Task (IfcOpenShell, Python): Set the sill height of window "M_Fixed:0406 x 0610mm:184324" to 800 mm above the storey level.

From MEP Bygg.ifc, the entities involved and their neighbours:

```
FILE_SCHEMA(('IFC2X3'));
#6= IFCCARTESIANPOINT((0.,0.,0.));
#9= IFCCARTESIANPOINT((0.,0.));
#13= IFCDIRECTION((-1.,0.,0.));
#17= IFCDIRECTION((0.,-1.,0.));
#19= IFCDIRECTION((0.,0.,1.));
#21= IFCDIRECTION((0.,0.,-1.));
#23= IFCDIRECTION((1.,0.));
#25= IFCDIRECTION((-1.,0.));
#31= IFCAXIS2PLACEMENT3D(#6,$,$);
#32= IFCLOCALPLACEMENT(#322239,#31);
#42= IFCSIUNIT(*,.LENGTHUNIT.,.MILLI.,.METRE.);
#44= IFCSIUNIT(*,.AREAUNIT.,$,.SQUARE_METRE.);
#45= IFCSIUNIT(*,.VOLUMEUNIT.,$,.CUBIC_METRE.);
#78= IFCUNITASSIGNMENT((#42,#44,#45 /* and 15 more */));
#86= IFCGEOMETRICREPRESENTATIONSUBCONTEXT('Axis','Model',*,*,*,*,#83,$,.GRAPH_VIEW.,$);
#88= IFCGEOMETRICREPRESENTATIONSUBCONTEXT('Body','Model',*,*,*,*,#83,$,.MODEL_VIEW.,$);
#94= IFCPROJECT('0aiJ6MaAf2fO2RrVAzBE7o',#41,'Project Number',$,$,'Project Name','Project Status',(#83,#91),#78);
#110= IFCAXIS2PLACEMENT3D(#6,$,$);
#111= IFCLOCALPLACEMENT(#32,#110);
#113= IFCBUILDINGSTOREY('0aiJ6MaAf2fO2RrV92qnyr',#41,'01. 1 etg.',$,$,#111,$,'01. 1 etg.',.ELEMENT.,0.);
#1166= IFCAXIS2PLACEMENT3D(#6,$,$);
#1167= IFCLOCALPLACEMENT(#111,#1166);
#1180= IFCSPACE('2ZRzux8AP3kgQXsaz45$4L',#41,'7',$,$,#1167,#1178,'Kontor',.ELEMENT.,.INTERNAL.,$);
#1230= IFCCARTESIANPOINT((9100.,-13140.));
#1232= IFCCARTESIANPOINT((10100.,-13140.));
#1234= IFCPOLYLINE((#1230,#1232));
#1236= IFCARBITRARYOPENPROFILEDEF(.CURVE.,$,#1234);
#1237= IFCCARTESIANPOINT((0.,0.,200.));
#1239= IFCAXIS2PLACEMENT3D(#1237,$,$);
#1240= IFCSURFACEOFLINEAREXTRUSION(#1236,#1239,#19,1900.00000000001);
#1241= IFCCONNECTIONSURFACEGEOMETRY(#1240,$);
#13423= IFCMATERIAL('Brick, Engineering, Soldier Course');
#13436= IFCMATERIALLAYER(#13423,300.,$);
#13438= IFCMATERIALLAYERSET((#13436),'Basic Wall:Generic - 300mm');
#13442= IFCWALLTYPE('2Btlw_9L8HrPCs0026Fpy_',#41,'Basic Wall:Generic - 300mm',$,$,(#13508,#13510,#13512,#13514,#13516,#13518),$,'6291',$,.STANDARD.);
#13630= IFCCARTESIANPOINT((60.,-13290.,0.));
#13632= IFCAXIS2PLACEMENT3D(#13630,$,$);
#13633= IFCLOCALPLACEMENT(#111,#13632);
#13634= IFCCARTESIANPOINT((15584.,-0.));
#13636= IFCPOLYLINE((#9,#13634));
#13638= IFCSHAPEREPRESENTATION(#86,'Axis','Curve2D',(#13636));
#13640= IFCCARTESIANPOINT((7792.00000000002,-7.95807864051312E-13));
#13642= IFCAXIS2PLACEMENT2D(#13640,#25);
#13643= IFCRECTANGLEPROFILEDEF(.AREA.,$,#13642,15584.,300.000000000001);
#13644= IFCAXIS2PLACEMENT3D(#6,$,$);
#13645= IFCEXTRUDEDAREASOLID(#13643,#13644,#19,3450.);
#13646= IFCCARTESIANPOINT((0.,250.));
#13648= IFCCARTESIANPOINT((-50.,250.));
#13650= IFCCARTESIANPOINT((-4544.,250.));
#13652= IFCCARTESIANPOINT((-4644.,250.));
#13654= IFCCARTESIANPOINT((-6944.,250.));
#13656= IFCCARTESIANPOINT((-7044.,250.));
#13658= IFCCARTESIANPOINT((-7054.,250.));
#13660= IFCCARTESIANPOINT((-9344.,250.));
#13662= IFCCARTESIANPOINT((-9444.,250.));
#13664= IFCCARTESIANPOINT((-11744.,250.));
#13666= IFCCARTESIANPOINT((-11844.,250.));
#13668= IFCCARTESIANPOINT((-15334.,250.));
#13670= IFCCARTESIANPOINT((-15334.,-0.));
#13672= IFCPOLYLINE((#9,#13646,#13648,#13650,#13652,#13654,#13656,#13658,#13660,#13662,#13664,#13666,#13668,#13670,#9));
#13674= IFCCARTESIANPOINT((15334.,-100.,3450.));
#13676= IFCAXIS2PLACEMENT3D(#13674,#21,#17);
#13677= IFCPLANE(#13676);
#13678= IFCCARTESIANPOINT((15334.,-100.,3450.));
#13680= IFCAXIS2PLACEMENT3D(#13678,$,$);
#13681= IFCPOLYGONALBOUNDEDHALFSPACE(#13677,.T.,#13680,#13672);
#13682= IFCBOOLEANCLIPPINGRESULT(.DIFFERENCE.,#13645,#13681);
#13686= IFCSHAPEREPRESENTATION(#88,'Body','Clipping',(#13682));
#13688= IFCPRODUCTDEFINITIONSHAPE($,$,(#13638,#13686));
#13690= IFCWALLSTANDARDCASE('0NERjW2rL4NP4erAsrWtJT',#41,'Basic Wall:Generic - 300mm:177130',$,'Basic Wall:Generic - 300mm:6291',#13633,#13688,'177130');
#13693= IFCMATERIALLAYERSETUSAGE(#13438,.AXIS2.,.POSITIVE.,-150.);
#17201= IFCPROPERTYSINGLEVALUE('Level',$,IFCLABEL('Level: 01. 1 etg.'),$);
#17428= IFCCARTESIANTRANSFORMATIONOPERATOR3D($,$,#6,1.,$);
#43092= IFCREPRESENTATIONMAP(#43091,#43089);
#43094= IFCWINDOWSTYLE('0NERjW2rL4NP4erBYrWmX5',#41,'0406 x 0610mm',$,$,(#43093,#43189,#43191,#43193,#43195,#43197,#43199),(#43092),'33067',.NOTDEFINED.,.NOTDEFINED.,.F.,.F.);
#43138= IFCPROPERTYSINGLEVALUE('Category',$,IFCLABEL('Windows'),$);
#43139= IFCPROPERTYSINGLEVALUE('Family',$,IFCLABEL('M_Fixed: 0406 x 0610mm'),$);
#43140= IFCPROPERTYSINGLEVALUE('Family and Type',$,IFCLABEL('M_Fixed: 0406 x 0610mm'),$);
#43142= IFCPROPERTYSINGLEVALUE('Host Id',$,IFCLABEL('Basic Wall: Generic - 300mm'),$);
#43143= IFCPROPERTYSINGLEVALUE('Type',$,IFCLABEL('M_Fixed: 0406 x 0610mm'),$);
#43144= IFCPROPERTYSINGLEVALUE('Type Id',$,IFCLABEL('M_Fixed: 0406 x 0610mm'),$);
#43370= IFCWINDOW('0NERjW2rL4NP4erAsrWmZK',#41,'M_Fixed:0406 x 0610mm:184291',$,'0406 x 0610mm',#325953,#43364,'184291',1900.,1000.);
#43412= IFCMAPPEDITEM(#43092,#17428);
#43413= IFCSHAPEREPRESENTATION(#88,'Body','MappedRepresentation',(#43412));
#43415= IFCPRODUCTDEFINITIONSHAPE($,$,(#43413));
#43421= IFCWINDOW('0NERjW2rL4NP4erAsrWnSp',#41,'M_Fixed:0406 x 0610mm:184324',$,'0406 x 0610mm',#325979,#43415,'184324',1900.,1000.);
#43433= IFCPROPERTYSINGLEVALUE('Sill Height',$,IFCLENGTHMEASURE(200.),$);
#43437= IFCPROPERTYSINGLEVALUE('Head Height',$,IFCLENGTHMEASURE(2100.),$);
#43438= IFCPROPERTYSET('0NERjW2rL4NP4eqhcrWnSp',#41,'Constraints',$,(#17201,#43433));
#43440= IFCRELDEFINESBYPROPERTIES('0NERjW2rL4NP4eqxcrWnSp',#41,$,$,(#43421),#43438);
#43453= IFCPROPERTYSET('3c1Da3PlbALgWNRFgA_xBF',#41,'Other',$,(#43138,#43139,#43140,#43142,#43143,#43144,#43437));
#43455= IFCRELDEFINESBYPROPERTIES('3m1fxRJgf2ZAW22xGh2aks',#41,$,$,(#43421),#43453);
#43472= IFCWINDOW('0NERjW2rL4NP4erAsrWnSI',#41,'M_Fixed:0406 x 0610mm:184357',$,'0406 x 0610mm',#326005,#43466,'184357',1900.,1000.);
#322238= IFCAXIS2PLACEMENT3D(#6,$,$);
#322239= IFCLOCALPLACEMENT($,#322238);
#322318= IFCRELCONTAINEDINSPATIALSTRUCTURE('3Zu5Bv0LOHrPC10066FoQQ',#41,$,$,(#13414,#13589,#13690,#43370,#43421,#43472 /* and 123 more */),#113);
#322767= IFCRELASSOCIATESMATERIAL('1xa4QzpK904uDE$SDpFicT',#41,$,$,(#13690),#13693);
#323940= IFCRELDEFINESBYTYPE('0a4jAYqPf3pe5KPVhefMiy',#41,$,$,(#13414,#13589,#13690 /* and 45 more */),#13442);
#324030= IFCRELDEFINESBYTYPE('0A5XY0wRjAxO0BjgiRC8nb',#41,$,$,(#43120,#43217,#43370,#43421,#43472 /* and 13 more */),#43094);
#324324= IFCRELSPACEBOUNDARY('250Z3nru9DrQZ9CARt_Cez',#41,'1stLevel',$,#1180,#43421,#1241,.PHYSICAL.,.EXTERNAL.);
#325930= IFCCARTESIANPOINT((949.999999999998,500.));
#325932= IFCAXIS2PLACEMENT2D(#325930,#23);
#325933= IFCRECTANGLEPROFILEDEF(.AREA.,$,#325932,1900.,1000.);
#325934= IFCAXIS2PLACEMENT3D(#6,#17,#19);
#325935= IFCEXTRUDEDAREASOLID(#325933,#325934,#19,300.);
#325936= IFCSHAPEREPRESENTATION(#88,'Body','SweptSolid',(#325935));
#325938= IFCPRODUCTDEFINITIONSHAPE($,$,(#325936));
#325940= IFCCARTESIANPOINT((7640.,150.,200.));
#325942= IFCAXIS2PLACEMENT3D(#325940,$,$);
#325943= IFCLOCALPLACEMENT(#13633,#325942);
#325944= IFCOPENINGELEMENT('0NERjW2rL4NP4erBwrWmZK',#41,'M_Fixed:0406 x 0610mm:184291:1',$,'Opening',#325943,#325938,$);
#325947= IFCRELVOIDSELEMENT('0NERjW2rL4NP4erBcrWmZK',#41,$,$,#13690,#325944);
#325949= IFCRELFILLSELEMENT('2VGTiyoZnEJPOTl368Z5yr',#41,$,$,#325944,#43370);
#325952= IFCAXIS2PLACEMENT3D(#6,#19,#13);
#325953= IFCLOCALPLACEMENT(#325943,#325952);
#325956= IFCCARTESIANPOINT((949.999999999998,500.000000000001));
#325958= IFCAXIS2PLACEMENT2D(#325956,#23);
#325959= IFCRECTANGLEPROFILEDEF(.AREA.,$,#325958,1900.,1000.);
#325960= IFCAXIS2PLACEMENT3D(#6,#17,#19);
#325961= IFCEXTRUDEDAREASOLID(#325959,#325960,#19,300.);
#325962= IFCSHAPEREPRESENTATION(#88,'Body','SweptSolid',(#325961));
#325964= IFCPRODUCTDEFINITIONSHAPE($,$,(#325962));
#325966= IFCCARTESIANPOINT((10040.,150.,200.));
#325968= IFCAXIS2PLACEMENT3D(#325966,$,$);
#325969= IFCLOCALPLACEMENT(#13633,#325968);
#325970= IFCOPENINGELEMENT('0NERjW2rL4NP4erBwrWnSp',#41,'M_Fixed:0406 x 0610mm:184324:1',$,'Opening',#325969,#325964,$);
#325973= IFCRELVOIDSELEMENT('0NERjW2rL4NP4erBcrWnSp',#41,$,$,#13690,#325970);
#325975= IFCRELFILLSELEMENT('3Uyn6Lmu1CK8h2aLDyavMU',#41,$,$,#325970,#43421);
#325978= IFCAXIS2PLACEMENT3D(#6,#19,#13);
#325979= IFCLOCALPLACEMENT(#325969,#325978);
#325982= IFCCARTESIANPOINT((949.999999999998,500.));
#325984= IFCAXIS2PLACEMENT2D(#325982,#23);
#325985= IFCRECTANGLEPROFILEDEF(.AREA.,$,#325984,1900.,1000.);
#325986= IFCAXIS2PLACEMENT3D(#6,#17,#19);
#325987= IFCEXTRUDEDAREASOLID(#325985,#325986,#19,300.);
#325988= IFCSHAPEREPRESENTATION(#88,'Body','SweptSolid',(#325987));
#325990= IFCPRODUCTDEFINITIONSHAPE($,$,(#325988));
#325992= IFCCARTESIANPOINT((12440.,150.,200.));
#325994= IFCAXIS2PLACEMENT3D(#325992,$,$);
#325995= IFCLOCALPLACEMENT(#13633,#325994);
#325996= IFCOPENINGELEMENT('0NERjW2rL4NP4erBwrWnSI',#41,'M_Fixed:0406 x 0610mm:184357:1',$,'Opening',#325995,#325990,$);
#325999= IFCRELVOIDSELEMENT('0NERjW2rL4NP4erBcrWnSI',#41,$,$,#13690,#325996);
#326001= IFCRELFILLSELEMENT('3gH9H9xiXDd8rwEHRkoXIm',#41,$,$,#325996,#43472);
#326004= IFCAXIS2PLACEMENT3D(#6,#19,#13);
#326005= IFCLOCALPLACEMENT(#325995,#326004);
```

```python
import numpy as np
import ifcopenshell
import ifcopenshell.api.geometry
import ifcopenshell.api.pset
import ifcopenshell.geom
import ifcopenshell.util.element
import ifcopenshell.util.placement
import ifcopenshell.util.shape
import ifcopenshell.util.unit

model = ifcopenshell.open("MEP Bygg.ifc")
unit_scale = ifcopenshell.util.unit.calculate_unit_scale(model)

window = model.by_guid("0NERjW2rL4NP4erAsrWnSp")
opening = window.FillsVoids[0].RelatingOpeningElement
storey = ifcopenshell.util.element.get_container(window, ifc_class="IfcBuildingStorey")
level = ifcopenshell.util.placement.get_local_placement(storey.ObjectPlacement)[2, 3]

# The opening's origin need not be at the sill, so measure its lowest point.
shape = ifcopenshell.geom.create_shape(ifcopenshell.geom.settings(), opening)
bottom = ifcopenshell.util.shape.get_shape_bottom_elevation(shape, shape.geometry) / unit_scale
dz = level + 800.0 - bottom

shift = np.array([0.0, 0.0, dz])
# The window is placed relative to its opening, so it follows when the opening moves.
matrix = ifcopenshell.util.placement.get_local_placement(opening.ObjectPlacement)
matrix[:3, 3] += shift
ifcopenshell.api.geometry.edit_object_placement(
    model, product=opening, matrix=matrix, is_si=False, should_transform_children=True
)

# Space boundary surfaces are stored in each space's coordinates; move them too.
for rel in window.ProvidesBoundaries:
    if not rel.ConnectionGeometry:
        continue
    surface = rel.ConnectionGeometry.SurfaceOnRelatingElement
    space_matrix = ifcopenshell.util.placement.get_local_placement(rel.RelatingSpace.ObjectPlacement)
    point = np.array(surface.Position.Location.Coordinates) + space_matrix[:3, :3].T @ shift
    surface.Position = model.createIfcAxis2Placement3D(
        model.createIfcCartesianPoint(point.tolist()), surface.Position.Axis, surface.Position.RefDirection
    )

# Keep the stored heights in step.
pset = model.by_id(ifcopenshell.util.element.get_pset(window, "Constraints", should_inherit=False)["id"])
ifcopenshell.api.pset.edit_pset(model, pset=pset, properties={
    "Sill Height": model.create_entity("IfcLengthMeasure", ifcopenshell.util.element.get_pset(window, "Constraints", "Sill Height") + dz),
})
pset = model.by_id(ifcopenshell.util.element.get_pset(window, "Other", should_inherit=False)["id"])
ifcopenshell.api.pset.edit_pset(model, pset=pset, properties={
    "Head Height": model.create_entity("IfcLengthMeasure", ifcopenshell.util.element.get_pset(window, "Other", "Head Height") + dz),
})

print(f"moved by {dz * unit_scale:+.3f} m")

model.write("MEP Bygg_rev.ifc")
```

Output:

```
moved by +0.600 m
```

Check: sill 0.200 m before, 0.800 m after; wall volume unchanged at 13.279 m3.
